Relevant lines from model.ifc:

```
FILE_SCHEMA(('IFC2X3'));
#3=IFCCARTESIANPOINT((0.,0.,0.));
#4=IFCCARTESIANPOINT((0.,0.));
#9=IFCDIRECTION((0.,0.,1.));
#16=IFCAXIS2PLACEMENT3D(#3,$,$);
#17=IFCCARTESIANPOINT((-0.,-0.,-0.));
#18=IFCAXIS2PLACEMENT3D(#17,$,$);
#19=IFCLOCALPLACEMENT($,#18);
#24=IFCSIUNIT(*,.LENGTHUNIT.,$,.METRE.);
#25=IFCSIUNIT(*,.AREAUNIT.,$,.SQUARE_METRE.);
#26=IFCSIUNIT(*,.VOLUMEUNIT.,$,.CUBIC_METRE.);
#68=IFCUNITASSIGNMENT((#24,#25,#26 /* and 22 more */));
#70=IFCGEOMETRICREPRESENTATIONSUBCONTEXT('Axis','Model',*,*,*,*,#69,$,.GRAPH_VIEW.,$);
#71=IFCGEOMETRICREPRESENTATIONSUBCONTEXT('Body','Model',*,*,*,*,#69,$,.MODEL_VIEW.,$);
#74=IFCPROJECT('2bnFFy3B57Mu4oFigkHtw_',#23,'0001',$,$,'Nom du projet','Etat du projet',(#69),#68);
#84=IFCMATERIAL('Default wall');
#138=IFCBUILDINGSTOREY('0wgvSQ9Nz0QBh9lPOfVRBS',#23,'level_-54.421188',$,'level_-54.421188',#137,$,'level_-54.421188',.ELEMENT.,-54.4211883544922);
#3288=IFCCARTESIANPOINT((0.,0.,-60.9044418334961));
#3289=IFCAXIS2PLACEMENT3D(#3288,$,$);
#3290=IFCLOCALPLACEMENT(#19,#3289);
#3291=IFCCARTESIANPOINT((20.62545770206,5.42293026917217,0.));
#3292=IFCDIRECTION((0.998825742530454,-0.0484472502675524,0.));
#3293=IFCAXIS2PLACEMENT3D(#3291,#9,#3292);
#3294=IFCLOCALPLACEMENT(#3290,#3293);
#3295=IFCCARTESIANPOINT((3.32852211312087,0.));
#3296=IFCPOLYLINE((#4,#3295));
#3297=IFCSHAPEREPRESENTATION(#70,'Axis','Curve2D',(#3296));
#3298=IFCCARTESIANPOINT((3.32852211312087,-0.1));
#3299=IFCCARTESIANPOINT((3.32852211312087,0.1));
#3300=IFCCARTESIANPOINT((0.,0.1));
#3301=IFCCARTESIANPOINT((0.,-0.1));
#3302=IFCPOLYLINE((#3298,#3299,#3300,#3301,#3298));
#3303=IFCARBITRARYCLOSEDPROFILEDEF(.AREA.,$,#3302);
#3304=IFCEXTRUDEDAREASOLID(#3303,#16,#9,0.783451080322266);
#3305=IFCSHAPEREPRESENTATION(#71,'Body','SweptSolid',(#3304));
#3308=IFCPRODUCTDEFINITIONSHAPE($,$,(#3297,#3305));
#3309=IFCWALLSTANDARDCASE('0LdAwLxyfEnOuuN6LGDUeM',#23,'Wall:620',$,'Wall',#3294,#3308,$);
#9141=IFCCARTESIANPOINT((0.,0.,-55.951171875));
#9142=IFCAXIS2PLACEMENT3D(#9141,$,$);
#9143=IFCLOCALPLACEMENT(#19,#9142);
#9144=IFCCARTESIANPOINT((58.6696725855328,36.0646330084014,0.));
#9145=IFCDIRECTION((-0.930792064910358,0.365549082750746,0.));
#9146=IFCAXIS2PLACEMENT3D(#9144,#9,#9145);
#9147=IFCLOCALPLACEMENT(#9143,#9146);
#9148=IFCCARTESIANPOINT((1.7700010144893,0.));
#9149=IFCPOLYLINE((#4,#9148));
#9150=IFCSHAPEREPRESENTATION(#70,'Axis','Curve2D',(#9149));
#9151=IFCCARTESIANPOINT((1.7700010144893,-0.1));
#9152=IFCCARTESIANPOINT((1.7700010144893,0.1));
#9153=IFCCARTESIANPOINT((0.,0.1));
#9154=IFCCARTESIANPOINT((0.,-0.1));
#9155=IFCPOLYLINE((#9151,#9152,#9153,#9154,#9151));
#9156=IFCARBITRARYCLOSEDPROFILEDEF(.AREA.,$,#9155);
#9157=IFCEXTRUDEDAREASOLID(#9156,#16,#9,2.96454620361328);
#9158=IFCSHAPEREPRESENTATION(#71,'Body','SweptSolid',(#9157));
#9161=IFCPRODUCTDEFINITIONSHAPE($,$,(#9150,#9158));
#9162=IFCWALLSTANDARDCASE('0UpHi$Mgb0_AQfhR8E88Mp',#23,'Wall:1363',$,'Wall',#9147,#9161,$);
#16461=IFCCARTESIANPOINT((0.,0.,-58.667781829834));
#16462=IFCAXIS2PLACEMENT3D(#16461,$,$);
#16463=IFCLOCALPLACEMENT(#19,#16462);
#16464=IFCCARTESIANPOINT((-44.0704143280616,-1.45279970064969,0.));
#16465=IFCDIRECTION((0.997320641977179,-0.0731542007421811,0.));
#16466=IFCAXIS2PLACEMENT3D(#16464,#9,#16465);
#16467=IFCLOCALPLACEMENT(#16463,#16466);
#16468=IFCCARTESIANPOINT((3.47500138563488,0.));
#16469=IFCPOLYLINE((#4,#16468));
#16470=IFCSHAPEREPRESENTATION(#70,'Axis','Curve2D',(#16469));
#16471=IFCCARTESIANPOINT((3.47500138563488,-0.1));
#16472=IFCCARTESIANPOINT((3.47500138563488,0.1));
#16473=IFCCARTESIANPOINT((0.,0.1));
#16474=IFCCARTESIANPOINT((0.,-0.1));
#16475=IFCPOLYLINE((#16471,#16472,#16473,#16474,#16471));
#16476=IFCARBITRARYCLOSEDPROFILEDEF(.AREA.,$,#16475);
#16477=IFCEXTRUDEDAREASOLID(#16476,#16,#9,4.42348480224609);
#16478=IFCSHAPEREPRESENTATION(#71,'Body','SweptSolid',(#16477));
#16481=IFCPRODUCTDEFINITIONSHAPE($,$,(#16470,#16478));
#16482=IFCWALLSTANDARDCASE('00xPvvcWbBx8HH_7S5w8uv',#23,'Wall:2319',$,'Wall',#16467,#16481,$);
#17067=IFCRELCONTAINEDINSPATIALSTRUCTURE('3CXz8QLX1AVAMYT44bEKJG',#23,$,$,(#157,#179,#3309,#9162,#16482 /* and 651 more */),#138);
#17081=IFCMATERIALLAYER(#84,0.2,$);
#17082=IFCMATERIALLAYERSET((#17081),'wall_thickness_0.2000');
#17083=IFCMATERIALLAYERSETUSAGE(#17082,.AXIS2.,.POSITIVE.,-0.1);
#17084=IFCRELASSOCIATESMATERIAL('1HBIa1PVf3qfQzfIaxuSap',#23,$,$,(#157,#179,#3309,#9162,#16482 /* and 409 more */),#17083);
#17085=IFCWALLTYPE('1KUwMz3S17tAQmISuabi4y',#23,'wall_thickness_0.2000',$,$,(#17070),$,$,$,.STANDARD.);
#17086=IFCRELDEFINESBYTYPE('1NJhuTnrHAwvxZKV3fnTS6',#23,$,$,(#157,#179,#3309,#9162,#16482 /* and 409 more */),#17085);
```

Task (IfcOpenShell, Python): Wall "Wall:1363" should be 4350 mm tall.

```python
import ifcopenshell
import ifcopenshell.geom
import ifcopenshell.util.representation
import ifcopenshell.util.shape
import ifcopenshell.util.unit

model = ifcopenshell.open("model.ifc")
unit_scale = ifcopenshell.util.unit.calculate_unit_scale(model)
settings = ifcopenshell.geom.settings()


def volume(element):
    """Net volume in cubic metres, openings subtracted."""
    shape = ifcopenshell.geom.create_shape(settings, element)
    return ifcopenshell.util.shape.get_volume(shape.geometry)


wall = model.by_guid("0UpHi$Mgb0_AQfhR8E88Mp")
before = volume(wall)

body = ifcopenshell.util.representation.get_representation(wall, "Model", "Body")
solid = body.Items[0]
old_height = solid.Depth
solid.Depth = 4.35 / unit_scale
after = volume(wall)

print(f"height {old_height:g} -> {solid.Depth:g}, volume {before:.3f} -> {after:.3f} m3")

model.write("model_rev.ifc")
```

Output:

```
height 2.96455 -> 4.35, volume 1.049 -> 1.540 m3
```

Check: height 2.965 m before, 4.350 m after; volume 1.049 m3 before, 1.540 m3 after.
